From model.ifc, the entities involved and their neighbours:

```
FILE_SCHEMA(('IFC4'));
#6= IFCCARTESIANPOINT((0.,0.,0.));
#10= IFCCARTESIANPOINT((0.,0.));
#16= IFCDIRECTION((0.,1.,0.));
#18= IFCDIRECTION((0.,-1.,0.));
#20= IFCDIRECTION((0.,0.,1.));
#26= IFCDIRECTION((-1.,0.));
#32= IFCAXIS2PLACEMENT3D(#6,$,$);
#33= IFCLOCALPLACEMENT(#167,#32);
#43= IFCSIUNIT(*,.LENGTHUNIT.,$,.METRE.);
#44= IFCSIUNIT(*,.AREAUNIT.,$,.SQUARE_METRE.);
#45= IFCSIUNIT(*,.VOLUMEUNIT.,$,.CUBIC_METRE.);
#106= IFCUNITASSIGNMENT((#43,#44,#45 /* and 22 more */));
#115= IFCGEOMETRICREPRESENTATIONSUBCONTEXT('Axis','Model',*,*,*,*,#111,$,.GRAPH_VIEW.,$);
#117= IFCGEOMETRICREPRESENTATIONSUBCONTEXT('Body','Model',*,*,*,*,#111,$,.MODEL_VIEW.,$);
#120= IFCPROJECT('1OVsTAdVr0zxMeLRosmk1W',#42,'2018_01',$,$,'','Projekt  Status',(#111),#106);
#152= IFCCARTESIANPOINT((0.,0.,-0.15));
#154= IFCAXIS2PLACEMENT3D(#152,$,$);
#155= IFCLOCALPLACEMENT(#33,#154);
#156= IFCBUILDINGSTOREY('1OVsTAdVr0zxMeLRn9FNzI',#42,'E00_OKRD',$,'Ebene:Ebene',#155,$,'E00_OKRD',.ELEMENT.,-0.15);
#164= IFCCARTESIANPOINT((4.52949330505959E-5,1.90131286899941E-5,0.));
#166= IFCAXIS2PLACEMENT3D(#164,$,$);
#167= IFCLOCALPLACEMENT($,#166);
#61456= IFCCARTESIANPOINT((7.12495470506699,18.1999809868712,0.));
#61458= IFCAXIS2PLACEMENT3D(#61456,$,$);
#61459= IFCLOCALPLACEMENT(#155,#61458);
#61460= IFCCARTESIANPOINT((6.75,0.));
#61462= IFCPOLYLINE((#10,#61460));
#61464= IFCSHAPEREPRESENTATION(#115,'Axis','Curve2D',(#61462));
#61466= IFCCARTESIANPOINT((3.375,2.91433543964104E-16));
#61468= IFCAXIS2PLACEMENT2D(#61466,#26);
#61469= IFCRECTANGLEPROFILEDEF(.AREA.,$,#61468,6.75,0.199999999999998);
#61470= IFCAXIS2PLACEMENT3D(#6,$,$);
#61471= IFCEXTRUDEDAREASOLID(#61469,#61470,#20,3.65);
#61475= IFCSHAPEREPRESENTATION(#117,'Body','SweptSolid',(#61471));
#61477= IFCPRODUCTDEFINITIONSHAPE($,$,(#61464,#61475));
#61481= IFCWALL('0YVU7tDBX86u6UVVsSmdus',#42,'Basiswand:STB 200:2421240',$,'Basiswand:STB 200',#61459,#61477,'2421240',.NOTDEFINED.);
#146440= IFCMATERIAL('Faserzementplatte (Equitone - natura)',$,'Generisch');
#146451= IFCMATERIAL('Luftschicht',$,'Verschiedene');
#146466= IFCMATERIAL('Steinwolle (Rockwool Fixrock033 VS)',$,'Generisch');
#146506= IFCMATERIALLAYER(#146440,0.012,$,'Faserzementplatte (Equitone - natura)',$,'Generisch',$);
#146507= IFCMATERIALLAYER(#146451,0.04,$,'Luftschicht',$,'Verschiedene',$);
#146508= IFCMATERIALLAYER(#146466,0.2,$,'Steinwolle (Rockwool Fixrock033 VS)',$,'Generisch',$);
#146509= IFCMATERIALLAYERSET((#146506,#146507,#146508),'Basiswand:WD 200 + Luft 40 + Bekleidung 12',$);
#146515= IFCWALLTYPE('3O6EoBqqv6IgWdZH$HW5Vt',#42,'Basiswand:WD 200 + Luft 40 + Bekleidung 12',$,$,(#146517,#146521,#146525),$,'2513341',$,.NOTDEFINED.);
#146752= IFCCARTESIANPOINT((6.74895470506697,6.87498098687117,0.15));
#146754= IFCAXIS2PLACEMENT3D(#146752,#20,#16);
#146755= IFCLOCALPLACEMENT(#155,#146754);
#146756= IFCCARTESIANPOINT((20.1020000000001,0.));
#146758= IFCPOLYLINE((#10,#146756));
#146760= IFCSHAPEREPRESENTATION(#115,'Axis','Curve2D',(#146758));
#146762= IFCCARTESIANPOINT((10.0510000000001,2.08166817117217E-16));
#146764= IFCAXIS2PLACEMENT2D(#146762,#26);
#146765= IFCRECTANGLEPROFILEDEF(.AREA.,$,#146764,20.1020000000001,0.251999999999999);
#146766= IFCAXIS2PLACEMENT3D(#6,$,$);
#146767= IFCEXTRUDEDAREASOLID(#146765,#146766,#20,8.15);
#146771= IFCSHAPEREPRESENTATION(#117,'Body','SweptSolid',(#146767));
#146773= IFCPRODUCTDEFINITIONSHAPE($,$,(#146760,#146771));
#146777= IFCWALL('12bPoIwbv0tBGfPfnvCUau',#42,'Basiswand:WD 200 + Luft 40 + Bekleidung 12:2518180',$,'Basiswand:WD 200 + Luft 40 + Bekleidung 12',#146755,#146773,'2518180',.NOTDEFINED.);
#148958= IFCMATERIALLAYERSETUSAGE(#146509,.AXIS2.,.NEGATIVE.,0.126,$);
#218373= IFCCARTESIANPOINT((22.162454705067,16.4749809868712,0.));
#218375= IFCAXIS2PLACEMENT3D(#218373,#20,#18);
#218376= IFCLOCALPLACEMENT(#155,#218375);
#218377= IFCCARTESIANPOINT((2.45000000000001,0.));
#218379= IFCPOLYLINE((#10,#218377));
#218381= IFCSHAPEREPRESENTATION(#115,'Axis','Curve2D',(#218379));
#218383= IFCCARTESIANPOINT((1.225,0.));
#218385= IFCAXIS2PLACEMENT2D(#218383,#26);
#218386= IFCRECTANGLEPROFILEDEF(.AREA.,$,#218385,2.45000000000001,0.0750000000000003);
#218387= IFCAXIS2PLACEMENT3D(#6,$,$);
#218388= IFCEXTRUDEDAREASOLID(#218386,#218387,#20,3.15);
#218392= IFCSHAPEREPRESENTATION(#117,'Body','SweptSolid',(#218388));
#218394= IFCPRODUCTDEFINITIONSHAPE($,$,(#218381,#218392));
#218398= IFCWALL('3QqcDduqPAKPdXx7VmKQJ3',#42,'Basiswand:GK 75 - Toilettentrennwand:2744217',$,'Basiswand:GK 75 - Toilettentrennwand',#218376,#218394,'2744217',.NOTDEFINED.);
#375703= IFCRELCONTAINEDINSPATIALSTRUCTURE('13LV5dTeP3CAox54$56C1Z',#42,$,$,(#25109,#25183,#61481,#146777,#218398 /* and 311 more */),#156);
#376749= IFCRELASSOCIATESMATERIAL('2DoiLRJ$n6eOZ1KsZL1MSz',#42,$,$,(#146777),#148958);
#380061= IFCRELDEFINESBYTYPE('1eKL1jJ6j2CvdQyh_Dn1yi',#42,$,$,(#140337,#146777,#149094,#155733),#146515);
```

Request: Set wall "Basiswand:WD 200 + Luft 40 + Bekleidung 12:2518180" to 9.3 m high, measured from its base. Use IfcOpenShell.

```python
import ifcopenshell
import ifcopenshell.geom
import ifcopenshell.util.representation
import ifcopenshell.util.shape
import ifcopenshell.util.unit

model = ifcopenshell.open("model.ifc")
unit_scale = ifcopenshell.util.unit.calculate_unit_scale(model)
settings = ifcopenshell.geom.settings()


def volume(element):
    """Net volume in cubic metres, openings subtracted."""
    shape = ifcopenshell.geom.create_shape(settings, element)
    return ifcopenshell.util.shape.get_volume(shape.geometry)


wall = model.by_guid("12bPoIwbv0tBGfPfnvCUau")
before = volume(wall)

body = ifcopenshell.util.representation.get_representation(wall, "Model", "Body")
solid = body.Items[0]
old_height = solid.Depth
solid.Depth = 9.3 / unit_scale
after = volume(wall)

print(f"height {old_height:g} -> {solid.Depth:g}, volume {before:.3f} -> {after:.3f} m3")

model.write("model_edited.ifc")
```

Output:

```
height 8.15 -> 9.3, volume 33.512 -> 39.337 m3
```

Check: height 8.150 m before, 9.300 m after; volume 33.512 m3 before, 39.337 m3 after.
